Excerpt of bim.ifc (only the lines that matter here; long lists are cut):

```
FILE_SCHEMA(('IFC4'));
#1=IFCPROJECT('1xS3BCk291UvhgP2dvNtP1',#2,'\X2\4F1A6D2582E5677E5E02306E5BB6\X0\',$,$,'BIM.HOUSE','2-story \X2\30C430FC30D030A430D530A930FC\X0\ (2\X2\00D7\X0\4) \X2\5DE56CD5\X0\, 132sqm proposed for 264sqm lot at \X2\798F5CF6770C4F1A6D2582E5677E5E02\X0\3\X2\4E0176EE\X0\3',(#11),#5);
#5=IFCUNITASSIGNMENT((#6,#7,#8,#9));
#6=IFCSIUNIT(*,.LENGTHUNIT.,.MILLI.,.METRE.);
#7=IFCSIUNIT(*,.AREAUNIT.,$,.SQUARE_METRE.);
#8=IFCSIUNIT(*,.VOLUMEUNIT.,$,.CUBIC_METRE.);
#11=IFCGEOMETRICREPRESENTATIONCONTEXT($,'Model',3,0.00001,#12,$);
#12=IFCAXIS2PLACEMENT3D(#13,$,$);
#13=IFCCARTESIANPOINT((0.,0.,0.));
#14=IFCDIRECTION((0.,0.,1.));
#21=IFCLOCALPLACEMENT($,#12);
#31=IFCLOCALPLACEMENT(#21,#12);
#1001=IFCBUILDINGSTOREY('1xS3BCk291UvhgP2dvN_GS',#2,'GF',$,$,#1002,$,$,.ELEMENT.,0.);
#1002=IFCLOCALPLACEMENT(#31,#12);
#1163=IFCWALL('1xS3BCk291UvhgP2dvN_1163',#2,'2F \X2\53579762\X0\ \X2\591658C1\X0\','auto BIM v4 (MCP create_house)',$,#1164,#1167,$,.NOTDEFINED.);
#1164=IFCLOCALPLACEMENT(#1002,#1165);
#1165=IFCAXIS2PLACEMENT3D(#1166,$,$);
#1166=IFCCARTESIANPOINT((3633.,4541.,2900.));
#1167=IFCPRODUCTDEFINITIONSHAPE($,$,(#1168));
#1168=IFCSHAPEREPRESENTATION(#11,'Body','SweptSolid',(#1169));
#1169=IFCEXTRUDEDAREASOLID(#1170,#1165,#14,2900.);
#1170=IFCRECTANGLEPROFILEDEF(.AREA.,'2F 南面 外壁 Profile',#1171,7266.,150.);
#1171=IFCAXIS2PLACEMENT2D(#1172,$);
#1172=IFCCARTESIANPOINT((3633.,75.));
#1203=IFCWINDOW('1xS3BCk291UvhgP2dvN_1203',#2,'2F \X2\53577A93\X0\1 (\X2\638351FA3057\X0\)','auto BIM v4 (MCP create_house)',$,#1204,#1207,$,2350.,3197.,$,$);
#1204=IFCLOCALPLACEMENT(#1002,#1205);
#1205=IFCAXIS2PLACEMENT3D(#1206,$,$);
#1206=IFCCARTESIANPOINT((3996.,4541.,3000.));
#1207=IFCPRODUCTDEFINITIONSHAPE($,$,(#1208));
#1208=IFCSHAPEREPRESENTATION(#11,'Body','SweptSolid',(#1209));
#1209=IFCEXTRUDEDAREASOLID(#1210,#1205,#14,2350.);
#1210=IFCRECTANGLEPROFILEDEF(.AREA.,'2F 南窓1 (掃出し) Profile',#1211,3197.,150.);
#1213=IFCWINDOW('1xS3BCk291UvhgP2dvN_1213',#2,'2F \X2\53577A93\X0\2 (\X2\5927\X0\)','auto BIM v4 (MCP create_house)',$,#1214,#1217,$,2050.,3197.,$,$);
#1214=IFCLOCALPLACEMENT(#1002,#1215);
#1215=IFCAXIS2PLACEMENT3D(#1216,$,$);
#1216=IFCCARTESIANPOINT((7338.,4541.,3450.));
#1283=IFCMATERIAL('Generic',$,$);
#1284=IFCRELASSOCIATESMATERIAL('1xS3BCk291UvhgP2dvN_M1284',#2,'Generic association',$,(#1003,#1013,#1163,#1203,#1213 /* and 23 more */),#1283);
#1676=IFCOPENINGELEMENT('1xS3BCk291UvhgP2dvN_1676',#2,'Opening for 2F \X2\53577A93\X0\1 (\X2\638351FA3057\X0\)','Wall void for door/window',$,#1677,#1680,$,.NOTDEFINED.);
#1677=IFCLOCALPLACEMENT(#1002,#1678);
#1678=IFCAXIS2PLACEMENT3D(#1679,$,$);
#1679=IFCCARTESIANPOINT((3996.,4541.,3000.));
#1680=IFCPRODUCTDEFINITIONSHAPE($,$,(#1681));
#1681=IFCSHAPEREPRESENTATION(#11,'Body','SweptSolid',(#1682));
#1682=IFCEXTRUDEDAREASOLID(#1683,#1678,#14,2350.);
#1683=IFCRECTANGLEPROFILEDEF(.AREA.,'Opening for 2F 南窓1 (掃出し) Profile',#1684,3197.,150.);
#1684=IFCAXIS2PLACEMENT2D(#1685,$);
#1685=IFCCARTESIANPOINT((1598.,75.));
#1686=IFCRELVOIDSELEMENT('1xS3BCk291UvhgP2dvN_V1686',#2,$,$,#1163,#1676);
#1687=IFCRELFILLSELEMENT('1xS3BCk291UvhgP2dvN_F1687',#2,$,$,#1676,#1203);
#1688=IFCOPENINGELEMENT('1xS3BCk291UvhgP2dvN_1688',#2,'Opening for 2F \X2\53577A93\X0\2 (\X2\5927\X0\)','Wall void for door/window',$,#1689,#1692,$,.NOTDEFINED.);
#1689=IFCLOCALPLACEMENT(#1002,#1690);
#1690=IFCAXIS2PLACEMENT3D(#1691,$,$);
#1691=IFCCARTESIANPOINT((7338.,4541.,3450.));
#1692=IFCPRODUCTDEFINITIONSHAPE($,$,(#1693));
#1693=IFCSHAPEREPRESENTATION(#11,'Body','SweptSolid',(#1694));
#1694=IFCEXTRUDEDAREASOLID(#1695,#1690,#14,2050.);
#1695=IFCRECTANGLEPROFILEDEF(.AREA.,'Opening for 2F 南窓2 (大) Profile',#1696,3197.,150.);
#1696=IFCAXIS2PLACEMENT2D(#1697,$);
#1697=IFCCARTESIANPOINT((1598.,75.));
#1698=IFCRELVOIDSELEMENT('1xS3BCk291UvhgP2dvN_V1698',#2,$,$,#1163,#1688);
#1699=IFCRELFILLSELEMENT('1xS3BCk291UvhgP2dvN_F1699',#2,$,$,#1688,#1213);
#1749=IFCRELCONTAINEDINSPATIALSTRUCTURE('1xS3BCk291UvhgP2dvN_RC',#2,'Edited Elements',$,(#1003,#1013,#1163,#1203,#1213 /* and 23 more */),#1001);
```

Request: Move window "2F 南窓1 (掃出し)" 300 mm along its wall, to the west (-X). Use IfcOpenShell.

```python
import ifcopenshell
import ifcopenshell.api.geometry
import ifcopenshell.util.placement
import ifcopenshell.util.unit

model = ifcopenshell.open("bim.ifc")
unit_scale = ifcopenshell.util.unit.calculate_unit_scale(model)

window = model.by_guid("1xS3BCk291UvhgP2dvN_1203")
opening = window.FillsVoids[0].RelatingOpeningElement
wall = opening.VoidsElements[0].RelatingBuildingElement

wall_matrix = ifcopenshell.util.placement.get_local_placement(wall.ObjectPlacement)
shift = wall_matrix[:3, 0] * -0.3 / unit_scale
before = ifcopenshell.util.placement.get_local_placement(window.ObjectPlacement)[:3, 3].copy()

# The window is not placed relative to its opening, so move both.
for product in (opening, window):
    matrix = ifcopenshell.util.placement.get_local_placement(product.ObjectPlacement)
    matrix[:3, 3] += shift
    ifcopenshell.api.geometry.edit_object_placement(model, product=product, matrix=matrix, is_si=False)

after = ifcopenshell.util.placement.get_local_placement(window.ObjectPlacement)[:3, 3]
print("window moved by", (after - before).round(3) + 0.0)

model.write("bim_v2.ifc")
```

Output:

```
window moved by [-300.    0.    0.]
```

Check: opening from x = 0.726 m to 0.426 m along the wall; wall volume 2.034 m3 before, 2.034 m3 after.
